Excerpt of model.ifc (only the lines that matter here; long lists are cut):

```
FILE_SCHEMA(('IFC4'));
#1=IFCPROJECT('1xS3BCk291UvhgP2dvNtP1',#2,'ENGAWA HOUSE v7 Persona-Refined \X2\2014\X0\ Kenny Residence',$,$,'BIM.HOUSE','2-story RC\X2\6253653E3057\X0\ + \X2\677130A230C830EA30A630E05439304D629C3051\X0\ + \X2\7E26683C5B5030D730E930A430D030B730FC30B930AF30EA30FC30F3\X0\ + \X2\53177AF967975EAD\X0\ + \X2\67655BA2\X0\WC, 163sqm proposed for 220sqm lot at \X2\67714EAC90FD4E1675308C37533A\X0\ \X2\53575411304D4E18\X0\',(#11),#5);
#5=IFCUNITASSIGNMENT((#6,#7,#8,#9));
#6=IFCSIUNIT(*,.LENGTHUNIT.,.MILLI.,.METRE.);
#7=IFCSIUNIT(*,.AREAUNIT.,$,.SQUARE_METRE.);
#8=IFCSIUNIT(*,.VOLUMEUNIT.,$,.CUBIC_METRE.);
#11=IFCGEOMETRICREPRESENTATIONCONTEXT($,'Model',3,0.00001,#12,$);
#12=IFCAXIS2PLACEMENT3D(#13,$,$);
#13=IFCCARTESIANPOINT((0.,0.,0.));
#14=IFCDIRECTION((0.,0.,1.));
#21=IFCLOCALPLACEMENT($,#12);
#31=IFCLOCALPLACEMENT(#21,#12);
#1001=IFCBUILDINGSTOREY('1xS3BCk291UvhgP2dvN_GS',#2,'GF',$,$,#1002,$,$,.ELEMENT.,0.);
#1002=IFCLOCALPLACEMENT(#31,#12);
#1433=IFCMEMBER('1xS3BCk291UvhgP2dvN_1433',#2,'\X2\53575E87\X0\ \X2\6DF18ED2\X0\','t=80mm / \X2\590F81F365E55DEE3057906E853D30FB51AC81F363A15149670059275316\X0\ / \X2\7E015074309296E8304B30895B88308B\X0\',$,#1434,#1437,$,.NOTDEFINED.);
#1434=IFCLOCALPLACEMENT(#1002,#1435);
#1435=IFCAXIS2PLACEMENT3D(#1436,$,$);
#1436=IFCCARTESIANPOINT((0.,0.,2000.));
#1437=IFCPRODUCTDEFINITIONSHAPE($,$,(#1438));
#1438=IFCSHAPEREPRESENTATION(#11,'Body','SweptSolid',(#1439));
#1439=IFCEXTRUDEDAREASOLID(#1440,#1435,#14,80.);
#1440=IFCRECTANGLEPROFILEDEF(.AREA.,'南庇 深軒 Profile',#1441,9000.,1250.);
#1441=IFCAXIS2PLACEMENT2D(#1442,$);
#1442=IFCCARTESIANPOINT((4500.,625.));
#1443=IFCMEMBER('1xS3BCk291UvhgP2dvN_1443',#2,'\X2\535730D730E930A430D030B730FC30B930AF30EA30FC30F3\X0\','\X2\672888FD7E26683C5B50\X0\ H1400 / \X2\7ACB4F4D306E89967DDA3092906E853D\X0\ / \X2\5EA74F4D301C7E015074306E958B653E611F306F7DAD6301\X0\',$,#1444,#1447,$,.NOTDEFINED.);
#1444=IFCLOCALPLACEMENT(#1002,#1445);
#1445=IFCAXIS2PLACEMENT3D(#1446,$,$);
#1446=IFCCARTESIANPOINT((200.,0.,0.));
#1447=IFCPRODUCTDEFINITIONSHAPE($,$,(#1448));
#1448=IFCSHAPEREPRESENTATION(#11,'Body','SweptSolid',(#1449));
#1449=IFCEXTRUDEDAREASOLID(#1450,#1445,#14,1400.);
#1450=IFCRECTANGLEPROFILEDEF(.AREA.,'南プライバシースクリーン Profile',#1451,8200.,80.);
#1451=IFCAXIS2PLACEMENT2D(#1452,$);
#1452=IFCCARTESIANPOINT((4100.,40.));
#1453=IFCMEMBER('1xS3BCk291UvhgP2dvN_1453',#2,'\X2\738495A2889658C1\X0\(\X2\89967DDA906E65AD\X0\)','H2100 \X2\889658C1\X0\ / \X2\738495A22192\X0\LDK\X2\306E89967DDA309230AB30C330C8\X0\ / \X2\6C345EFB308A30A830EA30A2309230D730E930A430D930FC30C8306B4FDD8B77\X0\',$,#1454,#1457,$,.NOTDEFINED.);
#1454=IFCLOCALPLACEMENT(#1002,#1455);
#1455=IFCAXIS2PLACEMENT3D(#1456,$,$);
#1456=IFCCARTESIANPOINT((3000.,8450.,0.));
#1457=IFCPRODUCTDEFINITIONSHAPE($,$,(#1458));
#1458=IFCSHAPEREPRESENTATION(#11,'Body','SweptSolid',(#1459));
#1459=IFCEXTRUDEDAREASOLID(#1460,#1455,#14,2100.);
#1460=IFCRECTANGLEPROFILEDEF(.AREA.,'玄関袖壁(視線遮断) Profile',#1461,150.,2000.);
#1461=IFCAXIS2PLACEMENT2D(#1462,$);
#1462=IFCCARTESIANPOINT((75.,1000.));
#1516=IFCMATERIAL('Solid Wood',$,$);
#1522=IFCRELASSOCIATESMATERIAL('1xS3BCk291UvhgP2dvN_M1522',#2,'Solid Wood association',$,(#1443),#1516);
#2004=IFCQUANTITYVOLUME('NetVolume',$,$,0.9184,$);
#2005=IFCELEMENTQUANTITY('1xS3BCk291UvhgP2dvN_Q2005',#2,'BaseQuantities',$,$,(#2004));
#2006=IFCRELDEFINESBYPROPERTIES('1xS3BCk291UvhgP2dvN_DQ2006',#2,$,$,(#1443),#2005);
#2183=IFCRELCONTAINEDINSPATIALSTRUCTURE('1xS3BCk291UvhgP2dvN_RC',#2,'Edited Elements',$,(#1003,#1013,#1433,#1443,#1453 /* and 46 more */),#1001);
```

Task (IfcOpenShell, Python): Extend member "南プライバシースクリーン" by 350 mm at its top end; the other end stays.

```python
import ifcopenshell
import ifcopenshell.api.pset
import ifcopenshell.util.element

model = ifcopenshell.open("model.ifc")

member = model.by_guid("1xS3BCk291UvhgP2dvN_1443")
change = 350.0

# The extrusion runs towards the end named, so only its depth changes.
body = next(r for r in member.Representation.Representations if r.RepresentationIdentifier == "Body")
solid = body.Items[0]
old_length = solid.Depth
solid.Depth += change

# Update the stored length and volume.
qto = model.by_id(ifcopenshell.util.element.get_pset(member, "BaseQuantities", should_inherit=False)["id"])
ifcopenshell.api.pset.edit_qto(model, qto=qto, properties={
    "NetVolume": ifcopenshell.util.element.get_pset(member, "BaseQuantities", "NetVolume") * solid.Depth / old_length,
})

print(f"length {old_length:g} -> {solid.Depth:g}")

model.write("model_updated.ifc")
```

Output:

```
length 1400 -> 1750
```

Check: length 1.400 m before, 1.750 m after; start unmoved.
